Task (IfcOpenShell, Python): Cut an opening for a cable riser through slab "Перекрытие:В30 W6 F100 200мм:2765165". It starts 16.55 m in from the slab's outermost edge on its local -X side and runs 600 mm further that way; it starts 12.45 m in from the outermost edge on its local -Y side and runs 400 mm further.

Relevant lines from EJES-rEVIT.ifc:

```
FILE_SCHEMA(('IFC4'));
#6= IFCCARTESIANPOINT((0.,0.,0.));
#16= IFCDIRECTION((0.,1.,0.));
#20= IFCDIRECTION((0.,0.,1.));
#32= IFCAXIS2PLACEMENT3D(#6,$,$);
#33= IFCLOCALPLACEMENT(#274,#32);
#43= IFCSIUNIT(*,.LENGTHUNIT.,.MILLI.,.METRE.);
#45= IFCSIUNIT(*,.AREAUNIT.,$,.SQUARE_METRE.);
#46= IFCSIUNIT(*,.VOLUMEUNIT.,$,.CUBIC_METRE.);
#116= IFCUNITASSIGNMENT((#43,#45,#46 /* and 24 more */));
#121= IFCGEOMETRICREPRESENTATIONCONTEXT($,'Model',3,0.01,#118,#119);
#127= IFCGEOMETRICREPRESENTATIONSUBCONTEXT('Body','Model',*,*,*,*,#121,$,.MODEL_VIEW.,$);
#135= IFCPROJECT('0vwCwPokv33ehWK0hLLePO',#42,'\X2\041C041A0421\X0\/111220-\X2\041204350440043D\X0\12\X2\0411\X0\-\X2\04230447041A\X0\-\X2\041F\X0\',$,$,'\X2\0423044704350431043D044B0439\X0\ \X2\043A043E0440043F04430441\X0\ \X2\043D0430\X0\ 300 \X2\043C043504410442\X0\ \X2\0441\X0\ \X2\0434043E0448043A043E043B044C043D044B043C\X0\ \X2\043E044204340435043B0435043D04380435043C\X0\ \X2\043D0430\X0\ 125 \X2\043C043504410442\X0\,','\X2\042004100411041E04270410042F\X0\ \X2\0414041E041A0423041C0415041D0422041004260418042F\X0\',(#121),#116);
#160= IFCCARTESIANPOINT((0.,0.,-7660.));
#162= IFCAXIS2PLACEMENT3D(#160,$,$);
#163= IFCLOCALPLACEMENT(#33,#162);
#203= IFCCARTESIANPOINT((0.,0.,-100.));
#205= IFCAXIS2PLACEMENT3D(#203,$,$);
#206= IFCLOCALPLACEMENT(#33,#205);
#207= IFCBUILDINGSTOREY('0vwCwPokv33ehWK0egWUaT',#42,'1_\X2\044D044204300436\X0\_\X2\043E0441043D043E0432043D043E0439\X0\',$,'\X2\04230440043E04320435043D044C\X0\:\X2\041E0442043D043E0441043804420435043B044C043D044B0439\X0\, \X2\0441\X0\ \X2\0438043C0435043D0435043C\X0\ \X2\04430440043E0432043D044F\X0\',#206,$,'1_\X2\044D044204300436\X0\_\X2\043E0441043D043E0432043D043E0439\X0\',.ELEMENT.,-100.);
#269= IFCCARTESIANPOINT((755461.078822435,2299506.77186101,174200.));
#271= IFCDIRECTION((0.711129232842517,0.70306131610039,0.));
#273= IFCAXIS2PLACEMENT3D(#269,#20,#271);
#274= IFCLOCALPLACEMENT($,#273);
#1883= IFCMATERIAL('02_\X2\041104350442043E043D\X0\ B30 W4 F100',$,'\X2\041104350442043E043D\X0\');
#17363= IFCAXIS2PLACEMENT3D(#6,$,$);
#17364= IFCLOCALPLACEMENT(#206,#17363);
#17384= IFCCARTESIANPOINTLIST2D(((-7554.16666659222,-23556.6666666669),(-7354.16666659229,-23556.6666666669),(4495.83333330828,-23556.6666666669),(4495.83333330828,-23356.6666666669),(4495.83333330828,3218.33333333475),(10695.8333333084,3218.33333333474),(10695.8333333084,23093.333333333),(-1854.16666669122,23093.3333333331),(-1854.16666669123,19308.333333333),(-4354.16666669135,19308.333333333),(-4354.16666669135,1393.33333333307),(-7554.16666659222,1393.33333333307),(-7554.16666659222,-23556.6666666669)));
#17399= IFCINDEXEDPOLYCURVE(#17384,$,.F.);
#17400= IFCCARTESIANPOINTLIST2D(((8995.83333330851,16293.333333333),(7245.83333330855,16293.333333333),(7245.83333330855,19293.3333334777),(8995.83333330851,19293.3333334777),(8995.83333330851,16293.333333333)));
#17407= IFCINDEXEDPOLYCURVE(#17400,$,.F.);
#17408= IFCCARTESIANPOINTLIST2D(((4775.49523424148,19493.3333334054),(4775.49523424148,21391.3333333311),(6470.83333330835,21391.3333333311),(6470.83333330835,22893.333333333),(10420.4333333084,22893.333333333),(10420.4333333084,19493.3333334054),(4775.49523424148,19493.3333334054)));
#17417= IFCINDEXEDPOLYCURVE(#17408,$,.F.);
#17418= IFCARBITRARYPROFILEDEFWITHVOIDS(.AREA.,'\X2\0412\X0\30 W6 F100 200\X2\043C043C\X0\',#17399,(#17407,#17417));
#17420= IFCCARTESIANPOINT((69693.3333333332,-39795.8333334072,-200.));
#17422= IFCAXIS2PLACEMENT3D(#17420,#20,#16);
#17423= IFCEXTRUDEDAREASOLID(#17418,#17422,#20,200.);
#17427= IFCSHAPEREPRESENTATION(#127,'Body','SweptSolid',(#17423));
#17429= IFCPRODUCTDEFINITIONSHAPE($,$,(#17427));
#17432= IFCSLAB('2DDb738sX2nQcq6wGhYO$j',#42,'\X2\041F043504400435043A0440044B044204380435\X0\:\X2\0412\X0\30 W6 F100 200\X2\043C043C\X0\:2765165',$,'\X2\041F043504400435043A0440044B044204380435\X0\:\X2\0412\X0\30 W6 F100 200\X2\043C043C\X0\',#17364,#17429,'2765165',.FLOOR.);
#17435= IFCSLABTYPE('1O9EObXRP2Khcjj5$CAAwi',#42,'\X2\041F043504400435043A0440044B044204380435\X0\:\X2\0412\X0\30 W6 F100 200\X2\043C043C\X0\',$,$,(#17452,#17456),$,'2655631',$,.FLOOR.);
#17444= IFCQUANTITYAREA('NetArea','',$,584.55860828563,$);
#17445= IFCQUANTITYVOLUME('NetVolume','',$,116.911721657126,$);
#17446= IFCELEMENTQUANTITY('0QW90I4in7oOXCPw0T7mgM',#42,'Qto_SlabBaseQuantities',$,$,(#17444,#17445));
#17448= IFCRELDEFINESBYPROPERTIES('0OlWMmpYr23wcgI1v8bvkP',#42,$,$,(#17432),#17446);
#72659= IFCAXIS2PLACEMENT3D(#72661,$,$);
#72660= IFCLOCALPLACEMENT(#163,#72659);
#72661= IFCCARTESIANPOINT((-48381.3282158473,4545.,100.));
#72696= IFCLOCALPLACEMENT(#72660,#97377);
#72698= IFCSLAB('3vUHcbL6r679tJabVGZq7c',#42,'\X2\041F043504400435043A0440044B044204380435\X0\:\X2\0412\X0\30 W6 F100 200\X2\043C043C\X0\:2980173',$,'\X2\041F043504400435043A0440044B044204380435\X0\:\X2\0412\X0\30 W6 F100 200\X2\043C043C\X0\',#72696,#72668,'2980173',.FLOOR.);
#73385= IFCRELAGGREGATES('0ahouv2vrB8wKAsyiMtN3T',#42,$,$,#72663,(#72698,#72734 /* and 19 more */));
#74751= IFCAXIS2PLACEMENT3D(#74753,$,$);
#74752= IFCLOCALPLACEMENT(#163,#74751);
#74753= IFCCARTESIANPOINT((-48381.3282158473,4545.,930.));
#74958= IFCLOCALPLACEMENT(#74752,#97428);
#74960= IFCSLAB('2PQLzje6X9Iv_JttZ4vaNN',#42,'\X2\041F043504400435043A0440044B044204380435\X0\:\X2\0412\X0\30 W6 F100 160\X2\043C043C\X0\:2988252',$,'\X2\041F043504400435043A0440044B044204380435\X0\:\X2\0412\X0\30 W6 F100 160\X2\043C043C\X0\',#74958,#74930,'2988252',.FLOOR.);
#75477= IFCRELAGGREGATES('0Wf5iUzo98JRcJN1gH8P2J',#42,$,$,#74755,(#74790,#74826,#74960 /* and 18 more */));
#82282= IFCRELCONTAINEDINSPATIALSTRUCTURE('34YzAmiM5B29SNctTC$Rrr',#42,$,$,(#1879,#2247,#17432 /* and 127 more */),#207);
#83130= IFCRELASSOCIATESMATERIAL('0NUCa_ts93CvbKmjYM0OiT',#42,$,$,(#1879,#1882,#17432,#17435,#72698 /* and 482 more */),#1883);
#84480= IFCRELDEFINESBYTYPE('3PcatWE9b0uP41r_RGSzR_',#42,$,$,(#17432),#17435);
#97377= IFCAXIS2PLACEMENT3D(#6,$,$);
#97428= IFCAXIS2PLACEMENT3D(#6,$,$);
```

```python
import numpy as np
import ifcopenshell
import ifcopenshell.api.feature
import ifcopenshell.api.geometry
import ifcopenshell.api.pset
import ifcopenshell.api.root
import ifcopenshell.geom
import ifcopenshell.util.element
import ifcopenshell.util.placement
import ifcopenshell.util.representation
import ifcopenshell.util.shape
import ifcopenshell.util.unit

model = ifcopenshell.open("EJES-rEVIT.ifc")
unit_scale = ifcopenshell.util.unit.calculate_unit_scale(model)
area_scale = ifcopenshell.util.unit.calculate_unit_scale(model, "AREAUNIT")
volume_scale = ifcopenshell.util.unit.calculate_unit_scale(model, "VOLUMEUNIT")
settings = ifcopenshell.geom.settings()


def volume(element):
    """Net volume in cubic metres, openings subtracted."""
    shape = ifcopenshell.geom.create_shape(settings, element)
    return ifcopenshell.util.shape.get_volume(shape.geometry)


slab = model.by_id(17432)
before = volume(slab)

# Extent in the slab's own axes, in metres. The edges named are its -X and -Y sides.
slab_shape = ifcopenshell.geom.create_shape(settings, slab)
vertices = ifcopenshell.util.shape.get_vertices(slab_shape.geometry)
x_min, y_min, bottom = vertices.min(axis=0)
top = vertices[:, 2].max()

opening = ifcopenshell.api.root.create_entity(model, ifc_class="IfcOpeningElement", name="Cable riser opening", predefined_type="OPENING")
context = ifcopenshell.util.representation.get_context(model, "Model", "Body", "MODEL_VIEW")
width, depth = 0.6, 0.4
outline = [(0.0, 0.0), (width, 0.0), (width, depth), (0.0, depth), (0.0, 0.0)]
# Overshoot both faces by 50 mm so the cut is clean.
shape = ifcopenshell.api.geometry.add_slab_representation(
    model, context=context, depth=top - bottom + 0.1, polyline=outline
)
ifcopenshell.api.geometry.assign_representation(model, product=opening, representation=shape)

matrix = ifcopenshell.util.placement.get_local_placement(slab.ObjectPlacement)
matrix[:, 3] = matrix @ np.append(np.array([x_min + 16.55, y_min + 12.45, bottom - 0.05]) / unit_scale, 1.0)
ifcopenshell.api.geometry.edit_object_placement(model, product=opening, matrix=matrix, is_si=False)
ifcopenshell.api.feature.add_feature(model, feature=opening, element=slab)

after = volume(slab)

# Update the slab's stored quantities.
qto = model.by_id(ifcopenshell.util.element.get_pset(slab, "Qto_SlabBaseQuantities", should_inherit=False)["id"])
ifcopenshell.api.pset.edit_qto(model, qto=qto, properties={
    "NetArea": after / (top - bottom) / area_scale,
    "NetVolume": after / volume_scale,
})

print(f"slab volume {before:.3f} -> {after:.3f} m3")

model.write("EJES-rEVIT-out.ifc")
```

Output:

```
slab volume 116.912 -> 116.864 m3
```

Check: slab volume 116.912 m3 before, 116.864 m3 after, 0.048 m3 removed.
